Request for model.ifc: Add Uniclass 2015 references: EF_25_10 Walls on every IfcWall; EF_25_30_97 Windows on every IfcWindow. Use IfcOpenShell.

First a look at what the model holds.

```python
import ifcopenshell

model = ifcopenshell.open("model.ifc")
print(model.schema)
print("classifications:", [c.Name for c in model.by_type("IfcClassification")])
for ifc_class in ("IfcDoor", "IfcRoof", "IfcStair", "IfcWall", "IfcWindow"):
    print(ifc_class, len(model.by_type(ifc_class)))
```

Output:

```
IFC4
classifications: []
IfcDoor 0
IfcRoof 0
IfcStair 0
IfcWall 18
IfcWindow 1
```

```python
import ifcopenshell
import ifcopenshell.api.classification

model = ifcopenshell.open("model.ifc")

system = ifcopenshell.api.classification.add_classification(model, classification="Uniclass 2015")

codes = {
    "IfcWall": ("EF_25_10", "Walls"),
    "IfcWindow": ("EF_25_30_97", "Windows"),
}
for ifc_class, (code, name) in codes.items():
    products = model.by_type(ifc_class)
    ifcopenshell.api.classification.add_reference(
        model, products=products, classification=system, identification=code, name=name
    )
    print(code, len(products))

model.write("model_rev.ifc")
```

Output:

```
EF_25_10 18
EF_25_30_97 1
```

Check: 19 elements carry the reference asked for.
